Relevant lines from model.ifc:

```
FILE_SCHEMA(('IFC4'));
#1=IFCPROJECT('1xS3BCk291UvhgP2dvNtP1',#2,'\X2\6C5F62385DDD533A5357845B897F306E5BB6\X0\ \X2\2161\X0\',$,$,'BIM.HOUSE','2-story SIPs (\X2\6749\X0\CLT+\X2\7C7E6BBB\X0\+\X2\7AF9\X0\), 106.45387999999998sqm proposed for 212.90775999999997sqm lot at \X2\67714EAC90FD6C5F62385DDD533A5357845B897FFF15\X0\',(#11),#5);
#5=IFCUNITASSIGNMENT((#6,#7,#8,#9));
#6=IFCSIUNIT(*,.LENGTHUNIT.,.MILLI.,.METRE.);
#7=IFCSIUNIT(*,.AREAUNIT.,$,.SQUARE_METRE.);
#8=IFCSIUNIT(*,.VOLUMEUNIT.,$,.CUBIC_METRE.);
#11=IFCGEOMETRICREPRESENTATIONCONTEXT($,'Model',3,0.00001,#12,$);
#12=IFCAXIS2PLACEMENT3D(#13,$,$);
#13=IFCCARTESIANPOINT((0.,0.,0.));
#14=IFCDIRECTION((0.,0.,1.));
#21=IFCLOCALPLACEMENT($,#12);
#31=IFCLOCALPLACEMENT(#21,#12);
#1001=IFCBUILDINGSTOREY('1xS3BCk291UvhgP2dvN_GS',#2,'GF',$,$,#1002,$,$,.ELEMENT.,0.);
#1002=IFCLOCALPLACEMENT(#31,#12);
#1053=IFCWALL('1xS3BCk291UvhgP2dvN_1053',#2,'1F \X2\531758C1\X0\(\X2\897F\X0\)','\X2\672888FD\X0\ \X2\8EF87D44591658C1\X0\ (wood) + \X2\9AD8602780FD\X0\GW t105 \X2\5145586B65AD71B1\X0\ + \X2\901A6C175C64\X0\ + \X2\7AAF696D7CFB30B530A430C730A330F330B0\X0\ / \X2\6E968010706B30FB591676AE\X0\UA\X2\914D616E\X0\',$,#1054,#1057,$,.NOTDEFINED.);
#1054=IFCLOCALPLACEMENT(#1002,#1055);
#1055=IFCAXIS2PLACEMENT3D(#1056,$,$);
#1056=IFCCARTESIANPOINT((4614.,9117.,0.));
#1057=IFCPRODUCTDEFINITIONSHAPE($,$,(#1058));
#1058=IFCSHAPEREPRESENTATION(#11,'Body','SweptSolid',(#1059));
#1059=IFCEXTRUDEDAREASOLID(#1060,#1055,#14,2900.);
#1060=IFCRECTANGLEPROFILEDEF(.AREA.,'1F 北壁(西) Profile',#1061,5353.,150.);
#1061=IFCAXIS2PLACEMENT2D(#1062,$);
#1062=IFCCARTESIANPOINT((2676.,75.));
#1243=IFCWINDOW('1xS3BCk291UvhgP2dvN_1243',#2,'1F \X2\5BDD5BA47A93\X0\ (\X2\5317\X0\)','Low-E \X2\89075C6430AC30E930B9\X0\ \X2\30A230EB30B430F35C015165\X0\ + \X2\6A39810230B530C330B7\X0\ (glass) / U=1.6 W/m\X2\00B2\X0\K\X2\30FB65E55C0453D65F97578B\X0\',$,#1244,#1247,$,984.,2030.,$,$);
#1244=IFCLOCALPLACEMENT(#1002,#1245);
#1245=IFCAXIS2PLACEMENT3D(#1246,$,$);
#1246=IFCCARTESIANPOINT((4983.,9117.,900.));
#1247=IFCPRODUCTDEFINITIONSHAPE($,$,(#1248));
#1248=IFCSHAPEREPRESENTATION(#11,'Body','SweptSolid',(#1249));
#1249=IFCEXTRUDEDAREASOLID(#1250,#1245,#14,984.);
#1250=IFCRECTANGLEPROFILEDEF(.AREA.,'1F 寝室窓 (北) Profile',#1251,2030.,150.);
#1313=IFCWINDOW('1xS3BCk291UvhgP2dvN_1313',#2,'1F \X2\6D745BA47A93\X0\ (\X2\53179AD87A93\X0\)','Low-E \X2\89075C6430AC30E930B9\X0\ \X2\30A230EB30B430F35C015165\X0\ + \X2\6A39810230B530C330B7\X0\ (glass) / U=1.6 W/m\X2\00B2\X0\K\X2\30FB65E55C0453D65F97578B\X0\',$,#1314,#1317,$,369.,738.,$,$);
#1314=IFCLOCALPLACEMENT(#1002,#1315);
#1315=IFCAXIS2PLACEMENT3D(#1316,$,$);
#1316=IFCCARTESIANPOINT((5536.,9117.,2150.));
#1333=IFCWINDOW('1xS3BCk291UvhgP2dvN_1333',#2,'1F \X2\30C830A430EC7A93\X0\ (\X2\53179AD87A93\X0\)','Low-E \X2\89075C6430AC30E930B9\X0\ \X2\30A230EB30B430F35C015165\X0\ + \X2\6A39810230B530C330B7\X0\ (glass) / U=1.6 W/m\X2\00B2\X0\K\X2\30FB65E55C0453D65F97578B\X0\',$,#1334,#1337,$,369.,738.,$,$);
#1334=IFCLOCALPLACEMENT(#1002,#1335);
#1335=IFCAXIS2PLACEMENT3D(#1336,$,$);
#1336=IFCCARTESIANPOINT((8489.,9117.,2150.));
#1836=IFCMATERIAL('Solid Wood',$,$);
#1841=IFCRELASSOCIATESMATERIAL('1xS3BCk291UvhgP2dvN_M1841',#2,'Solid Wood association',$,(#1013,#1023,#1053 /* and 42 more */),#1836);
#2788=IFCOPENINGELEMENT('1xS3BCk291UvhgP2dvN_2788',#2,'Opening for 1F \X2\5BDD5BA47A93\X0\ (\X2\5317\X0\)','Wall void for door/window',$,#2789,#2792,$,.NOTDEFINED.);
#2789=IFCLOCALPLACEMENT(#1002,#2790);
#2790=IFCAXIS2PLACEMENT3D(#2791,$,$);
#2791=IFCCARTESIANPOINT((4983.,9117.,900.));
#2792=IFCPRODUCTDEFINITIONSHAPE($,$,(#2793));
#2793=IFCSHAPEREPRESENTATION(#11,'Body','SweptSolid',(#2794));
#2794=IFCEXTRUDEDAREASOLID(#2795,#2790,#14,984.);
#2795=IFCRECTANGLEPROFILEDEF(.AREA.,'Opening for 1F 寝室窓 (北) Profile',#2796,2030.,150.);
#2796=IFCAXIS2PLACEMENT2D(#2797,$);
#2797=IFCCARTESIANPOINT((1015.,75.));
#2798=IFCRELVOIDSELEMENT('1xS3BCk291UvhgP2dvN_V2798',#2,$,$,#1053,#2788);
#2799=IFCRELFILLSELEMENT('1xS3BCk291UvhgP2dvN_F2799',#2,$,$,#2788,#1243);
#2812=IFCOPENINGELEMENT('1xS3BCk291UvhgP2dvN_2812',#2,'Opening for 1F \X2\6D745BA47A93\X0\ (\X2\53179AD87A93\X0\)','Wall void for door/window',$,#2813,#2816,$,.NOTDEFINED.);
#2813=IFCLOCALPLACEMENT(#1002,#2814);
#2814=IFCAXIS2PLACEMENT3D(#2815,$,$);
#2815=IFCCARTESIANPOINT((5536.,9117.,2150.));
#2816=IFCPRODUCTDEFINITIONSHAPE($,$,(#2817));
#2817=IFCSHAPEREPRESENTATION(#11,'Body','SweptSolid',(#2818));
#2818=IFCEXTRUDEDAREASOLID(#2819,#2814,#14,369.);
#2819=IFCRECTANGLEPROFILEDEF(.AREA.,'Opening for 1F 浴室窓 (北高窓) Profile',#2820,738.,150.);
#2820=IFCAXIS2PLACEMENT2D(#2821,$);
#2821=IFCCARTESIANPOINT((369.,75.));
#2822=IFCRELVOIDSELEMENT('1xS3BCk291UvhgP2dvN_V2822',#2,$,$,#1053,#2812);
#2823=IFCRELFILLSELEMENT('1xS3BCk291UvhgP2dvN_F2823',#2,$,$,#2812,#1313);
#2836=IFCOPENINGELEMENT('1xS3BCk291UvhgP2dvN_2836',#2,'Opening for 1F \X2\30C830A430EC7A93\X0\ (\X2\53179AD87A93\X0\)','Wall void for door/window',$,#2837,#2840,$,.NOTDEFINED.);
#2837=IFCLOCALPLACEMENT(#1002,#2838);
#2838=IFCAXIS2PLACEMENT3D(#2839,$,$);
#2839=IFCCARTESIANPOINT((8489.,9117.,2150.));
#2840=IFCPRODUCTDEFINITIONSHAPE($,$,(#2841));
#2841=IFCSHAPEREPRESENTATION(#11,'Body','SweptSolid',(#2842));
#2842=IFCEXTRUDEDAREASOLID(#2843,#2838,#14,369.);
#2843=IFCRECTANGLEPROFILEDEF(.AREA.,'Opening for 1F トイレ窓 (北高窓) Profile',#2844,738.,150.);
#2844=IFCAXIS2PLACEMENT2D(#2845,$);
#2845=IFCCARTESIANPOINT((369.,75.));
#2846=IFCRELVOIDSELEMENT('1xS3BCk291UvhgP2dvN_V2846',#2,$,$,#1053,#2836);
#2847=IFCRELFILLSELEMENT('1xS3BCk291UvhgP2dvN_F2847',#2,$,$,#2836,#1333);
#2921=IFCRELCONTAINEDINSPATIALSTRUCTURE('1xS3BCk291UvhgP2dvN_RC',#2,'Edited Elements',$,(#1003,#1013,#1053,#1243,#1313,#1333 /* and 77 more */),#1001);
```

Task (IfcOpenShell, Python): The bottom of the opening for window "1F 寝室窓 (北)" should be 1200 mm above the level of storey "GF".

```python
import numpy as np
import ifcopenshell
import ifcopenshell.api.geometry
import ifcopenshell.geom
import ifcopenshell.util.element
import ifcopenshell.util.placement
import ifcopenshell.util.shape
import ifcopenshell.util.unit

model = ifcopenshell.open("model.ifc")
unit_scale = ifcopenshell.util.unit.calculate_unit_scale(model)

window = model.by_guid("1xS3BCk291UvhgP2dvN_1243")
opening = window.FillsVoids[0].RelatingOpeningElement
storey = ifcopenshell.util.element.get_container(window, ifc_class="IfcBuildingStorey")
level = ifcopenshell.util.placement.get_local_placement(storey.ObjectPlacement)[2, 3]

# The opening's origin need not be at the sill, so measure its lowest point.
shape = ifcopenshell.geom.create_shape(ifcopenshell.geom.settings(), opening)
bottom = ifcopenshell.util.shape.get_shape_bottom_elevation(shape, shape.geometry) / unit_scale
dz = level + 1.2 / unit_scale - bottom

shift = np.array([0.0, 0.0, dz])
# The window is not placed relative to its opening, so move both.
for product in (opening, window):
    matrix = ifcopenshell.util.placement.get_local_placement(product.ObjectPlacement)
    matrix[:3, 3] += shift
    ifcopenshell.api.geometry.edit_object_placement(model, product=product, matrix=matrix, is_si=False)

print(f"moved by {dz * unit_scale:+.3f} m")

model.write("model-out.ifc")
```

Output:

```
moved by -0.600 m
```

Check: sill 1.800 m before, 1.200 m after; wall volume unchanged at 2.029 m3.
